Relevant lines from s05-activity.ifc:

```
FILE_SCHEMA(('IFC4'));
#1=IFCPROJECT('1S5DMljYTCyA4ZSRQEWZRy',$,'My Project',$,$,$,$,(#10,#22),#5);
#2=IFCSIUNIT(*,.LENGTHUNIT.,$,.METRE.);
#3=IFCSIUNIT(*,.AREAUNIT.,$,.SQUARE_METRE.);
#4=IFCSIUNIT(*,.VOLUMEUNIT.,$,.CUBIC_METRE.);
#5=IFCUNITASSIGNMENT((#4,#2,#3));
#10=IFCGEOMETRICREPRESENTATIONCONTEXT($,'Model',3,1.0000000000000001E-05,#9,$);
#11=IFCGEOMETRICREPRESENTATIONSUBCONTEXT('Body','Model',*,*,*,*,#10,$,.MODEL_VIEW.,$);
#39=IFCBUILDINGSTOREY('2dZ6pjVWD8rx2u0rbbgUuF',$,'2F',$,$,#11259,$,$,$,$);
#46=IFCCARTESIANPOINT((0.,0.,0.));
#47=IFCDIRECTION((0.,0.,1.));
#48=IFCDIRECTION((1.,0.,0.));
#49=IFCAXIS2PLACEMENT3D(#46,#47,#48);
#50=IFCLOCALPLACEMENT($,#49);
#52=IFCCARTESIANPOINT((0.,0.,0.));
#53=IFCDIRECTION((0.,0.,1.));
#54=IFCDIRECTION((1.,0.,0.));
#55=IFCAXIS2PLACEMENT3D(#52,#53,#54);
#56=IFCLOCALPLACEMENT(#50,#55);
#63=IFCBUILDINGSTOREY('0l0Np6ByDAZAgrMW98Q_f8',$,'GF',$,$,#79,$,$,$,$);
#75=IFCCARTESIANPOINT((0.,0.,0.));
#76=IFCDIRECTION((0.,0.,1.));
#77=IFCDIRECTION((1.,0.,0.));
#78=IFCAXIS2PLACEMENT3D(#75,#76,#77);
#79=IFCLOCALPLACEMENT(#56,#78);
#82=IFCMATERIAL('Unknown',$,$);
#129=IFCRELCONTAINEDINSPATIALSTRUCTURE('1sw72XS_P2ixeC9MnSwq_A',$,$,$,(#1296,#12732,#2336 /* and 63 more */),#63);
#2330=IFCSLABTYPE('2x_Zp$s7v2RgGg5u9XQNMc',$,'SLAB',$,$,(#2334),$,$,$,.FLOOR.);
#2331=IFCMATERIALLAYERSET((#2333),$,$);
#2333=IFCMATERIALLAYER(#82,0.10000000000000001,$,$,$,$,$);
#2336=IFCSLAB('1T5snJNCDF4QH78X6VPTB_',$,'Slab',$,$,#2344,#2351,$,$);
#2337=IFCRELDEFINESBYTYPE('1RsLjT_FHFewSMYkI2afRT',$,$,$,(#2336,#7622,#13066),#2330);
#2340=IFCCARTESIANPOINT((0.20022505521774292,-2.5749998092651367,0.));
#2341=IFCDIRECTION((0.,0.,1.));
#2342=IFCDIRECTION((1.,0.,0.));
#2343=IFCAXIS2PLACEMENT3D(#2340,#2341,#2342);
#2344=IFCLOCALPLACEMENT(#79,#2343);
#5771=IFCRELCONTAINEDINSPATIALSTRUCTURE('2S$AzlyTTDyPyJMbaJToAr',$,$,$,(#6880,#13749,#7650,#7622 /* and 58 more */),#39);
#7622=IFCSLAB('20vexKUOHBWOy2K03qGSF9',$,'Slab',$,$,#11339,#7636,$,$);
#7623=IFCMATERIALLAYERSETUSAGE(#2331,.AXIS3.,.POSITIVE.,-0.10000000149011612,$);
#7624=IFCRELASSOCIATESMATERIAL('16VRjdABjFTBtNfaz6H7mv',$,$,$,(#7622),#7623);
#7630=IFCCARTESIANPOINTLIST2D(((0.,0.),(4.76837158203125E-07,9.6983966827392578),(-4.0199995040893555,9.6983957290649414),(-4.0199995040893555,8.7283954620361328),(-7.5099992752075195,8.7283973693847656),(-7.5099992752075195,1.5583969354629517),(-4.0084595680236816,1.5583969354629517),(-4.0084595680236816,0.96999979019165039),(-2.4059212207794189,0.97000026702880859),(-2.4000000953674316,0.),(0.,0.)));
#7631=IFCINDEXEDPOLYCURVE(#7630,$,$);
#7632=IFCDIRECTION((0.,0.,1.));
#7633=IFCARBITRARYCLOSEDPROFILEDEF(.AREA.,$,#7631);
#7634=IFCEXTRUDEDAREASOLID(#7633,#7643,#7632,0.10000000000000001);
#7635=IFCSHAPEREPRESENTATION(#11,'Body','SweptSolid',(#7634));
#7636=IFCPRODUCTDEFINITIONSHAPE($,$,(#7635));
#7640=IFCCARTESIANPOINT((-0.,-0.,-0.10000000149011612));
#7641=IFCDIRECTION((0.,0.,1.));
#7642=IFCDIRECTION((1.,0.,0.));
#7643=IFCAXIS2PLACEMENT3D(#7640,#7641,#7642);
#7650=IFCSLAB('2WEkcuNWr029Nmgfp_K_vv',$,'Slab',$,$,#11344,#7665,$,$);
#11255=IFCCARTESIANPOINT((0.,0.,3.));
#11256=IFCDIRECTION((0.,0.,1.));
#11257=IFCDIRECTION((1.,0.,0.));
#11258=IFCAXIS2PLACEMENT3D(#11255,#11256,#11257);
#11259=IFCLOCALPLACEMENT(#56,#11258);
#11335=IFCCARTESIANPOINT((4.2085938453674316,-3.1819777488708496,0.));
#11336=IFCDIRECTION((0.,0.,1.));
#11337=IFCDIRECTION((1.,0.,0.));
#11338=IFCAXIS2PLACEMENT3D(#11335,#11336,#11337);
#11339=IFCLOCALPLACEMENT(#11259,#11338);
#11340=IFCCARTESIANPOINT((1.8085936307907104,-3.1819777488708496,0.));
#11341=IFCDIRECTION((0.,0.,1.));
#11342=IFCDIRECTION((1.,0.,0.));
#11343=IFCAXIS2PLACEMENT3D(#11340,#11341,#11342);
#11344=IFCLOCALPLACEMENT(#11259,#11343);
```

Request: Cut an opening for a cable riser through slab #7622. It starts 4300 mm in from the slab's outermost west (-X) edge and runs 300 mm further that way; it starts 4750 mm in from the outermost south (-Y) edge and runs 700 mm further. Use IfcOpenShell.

```python
import numpy as np
import ifcopenshell
import ifcopenshell.api.feature
import ifcopenshell.api.geometry
import ifcopenshell.api.root
import ifcopenshell.geom
import ifcopenshell.util.placement
import ifcopenshell.util.representation
import ifcopenshell.util.shape
import ifcopenshell.util.unit

model = ifcopenshell.open("s05-activity.ifc")
unit_scale = ifcopenshell.util.unit.calculate_unit_scale(model)
settings = ifcopenshell.geom.settings()


def volume(element):
    """Net volume in cubic metres, openings subtracted."""
    shape = ifcopenshell.geom.create_shape(settings, element)
    return ifcopenshell.util.shape.get_volume(shape.geometry)


slab = model.by_guid("20vexKUOHBWOy2K03qGSF9")
before = volume(slab)

# Extent in the slab's own axes, in metres. The edges named are its -X and -Y sides.
slab_shape = ifcopenshell.geom.create_shape(settings, slab)
vertices = ifcopenshell.util.shape.get_vertices(slab_shape.geometry)
x_min, y_min, bottom = vertices.min(axis=0)
top = vertices[:, 2].max()

opening = ifcopenshell.api.root.create_entity(model, ifc_class="IfcOpeningElement", name="Cable riser opening", predefined_type="OPENING")
context = ifcopenshell.util.representation.get_context(model, "Model", "Body", "MODEL_VIEW")
width, depth = 0.3, 0.7
outline = [(0.0, 0.0), (width, 0.0), (width, depth), (0.0, depth), (0.0, 0.0)]
# Overshoot both faces by 50 mm so the cut is clean.
shape = ifcopenshell.api.geometry.add_slab_representation(
    model, context=context, depth=top - bottom + 0.1, polyline=outline
)
ifcopenshell.api.geometry.assign_representation(model, product=opening, representation=shape)

matrix = ifcopenshell.util.placement.get_local_placement(slab.ObjectPlacement)
matrix[:, 3] = matrix @ np.append(np.array([x_min + 4.3, y_min + 4.75, bottom - 0.05]) / unit_scale, 1.0)
ifcopenshell.api.geometry.edit_object_placement(model, product=opening, matrix=matrix, is_si=False)
ifcopenshell.api.feature.add_feature(model, feature=opening, element=slab)

after = volume(slab)

print(f"slab volume {before:.3f} -> {after:.3f} m3")

model.write("s05-activity_edited.ifc")
```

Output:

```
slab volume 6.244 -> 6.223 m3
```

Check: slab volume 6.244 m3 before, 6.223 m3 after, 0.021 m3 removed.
